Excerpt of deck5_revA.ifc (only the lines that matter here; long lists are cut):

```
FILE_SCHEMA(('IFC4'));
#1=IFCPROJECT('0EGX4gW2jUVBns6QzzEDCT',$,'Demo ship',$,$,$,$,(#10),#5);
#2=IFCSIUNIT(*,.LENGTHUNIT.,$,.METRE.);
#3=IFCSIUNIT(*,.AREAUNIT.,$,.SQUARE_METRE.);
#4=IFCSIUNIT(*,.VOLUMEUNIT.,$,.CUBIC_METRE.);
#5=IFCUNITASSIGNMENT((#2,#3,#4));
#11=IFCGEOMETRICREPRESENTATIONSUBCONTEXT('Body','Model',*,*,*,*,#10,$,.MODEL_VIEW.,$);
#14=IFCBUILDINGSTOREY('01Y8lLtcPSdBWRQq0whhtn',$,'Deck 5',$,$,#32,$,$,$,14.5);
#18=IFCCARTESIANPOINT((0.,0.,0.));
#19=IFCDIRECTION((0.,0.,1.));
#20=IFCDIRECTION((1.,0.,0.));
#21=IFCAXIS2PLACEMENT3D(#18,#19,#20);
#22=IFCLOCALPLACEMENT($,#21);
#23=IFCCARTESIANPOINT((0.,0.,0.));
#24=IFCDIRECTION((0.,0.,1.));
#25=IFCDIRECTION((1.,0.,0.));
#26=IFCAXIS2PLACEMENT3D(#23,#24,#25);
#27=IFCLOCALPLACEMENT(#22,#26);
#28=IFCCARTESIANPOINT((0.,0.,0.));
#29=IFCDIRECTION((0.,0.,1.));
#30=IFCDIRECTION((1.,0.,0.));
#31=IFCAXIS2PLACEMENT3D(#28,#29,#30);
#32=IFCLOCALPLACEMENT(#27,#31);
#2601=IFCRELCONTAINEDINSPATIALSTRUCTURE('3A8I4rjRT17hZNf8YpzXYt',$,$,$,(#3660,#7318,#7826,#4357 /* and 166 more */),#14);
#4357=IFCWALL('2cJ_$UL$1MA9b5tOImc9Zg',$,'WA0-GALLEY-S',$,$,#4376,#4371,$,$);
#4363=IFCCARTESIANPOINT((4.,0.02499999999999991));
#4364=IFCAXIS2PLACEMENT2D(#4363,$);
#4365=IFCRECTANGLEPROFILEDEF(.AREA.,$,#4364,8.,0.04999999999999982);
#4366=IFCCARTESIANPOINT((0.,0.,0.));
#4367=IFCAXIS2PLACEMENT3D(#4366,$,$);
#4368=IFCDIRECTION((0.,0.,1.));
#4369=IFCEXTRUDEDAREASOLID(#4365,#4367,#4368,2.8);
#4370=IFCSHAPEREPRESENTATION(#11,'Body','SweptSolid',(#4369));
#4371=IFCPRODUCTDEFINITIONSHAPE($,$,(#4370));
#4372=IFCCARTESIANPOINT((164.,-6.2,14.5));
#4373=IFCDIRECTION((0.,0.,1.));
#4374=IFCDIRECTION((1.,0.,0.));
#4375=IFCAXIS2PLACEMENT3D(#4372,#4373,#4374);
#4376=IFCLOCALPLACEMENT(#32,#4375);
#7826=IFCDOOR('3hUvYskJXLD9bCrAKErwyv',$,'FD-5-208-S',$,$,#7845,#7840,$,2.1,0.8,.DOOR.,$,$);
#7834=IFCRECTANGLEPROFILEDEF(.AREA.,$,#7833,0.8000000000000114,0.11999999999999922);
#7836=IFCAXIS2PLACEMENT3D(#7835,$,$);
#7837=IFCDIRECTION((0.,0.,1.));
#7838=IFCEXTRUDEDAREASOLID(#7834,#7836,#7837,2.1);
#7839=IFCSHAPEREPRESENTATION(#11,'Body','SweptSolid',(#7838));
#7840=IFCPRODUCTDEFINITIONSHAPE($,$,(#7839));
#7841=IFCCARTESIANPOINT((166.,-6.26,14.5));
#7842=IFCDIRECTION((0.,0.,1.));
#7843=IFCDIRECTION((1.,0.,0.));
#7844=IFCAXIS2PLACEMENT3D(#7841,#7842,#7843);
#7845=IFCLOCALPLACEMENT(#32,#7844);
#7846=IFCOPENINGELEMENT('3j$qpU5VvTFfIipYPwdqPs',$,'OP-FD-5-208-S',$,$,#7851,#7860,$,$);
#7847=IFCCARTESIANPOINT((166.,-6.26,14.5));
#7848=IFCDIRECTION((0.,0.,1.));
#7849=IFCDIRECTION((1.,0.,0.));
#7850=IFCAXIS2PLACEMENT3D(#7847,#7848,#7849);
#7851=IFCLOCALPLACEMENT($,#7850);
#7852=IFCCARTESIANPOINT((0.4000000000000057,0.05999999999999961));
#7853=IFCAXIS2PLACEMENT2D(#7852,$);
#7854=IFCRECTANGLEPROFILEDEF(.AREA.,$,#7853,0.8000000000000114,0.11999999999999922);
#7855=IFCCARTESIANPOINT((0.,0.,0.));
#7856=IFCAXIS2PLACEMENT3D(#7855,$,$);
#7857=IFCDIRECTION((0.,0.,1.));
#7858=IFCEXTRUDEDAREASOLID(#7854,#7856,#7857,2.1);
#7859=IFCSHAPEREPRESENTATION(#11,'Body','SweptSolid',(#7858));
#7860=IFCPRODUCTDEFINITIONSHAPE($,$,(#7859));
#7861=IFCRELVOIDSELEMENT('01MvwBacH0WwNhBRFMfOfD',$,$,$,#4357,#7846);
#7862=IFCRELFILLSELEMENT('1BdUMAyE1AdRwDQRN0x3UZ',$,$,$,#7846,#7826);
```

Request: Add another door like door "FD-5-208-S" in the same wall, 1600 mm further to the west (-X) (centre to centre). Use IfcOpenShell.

```python
import ifcopenshell
import ifcopenshell.api.feature
import ifcopenshell.api.geometry
import ifcopenshell.api.root
import ifcopenshell.geom
import ifcopenshell.util.element
import ifcopenshell.util.placement
import ifcopenshell.util.shape
import ifcopenshell.util.unit

model = ifcopenshell.open("deck5_revA.ifc")
unit_scale = ifcopenshell.util.unit.calculate_unit_scale(model)
settings = ifcopenshell.geom.settings()


def volume(element):
    """Net volume in cubic metres, openings subtracted."""
    shape = ifcopenshell.geom.create_shape(settings, element)
    return ifcopenshell.util.shape.get_volume(shape.geometry)


door = model.by_guid("3hUvYskJXLD9bCrAKErwyv")
opening = door.FillsVoids[0].RelatingOpeningElement
wall = opening.VoidsElements[0].RelatingBuildingElement
before = volume(wall)
shift = ifcopenshell.util.placement.get_local_placement(wall.ObjectPlacement)[:3, 0] * -1.6 / unit_scale

# copy_class copies the void relationship, type, container and properties, but no geometry.
new_opening = ifcopenshell.api.root.copy_class(model, product=opening)
new_opening.Representation = ifcopenshell.util.element.copy_deep(
    model, opening.Representation, exclude=["IfcGeometricRepresentationContext", "IfcRepresentationMap"]
)
new_door = ifcopenshell.api.root.copy_class(model, product=door)
new_door.Representation = ifcopenshell.util.element.copy_deep(
    model, door.Representation, exclude=["IfcGeometricRepresentationContext", "IfcRepresentationMap"]
)
ifcopenshell.api.feature.add_filling(model, opening=new_opening, element=new_door)

for old, new in ((opening, new_opening), (door, new_door)):
    matrix = ifcopenshell.util.placement.get_local_placement(old.ObjectPlacement)
    matrix[:3, 3] += shift
    ifcopenshell.api.geometry.edit_object_placement(model, product=new, matrix=matrix, is_si=False)

after = volume(wall)

print(f"wall volume {before:.3f} -> {after:.3f} m3")

model.write("deck5_revA-out.ifc")
```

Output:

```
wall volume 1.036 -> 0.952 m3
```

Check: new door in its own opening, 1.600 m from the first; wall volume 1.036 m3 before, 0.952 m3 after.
